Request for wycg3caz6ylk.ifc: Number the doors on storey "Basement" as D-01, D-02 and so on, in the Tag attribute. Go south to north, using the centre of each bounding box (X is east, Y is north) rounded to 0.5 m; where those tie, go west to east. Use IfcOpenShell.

First a look at what the model holds.

```python
import ifcopenshell
import ifcopenshell.util.element
import ifcopenshell.util.placement

model = ifcopenshell.open("wycg3caz6ylk.ifc")
print(model.schema)
storey = next(s for s in model.by_type("IfcBuildingStorey") if s.Name == "Basement")
doors = [e for e in ifcopenshell.util.element.get_decomposition(storey) if e.is_a("IfcDoor")]
for e in sorted(doors, key=lambda e: e.id()):
    origin = ifcopenshell.util.placement.get_local_placement(e.ObjectPlacement)[:3, 3]
    print(e.id(), e.Tag, e.Name, origin.round(2) + 0.0, sep=" | ")
```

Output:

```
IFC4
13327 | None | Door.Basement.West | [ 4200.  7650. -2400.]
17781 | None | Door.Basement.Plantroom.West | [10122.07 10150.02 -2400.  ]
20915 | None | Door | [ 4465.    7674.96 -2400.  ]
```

```python
import ifcopenshell
import ifcopenshell.geom
import ifcopenshell.util.element
import ifcopenshell.util.shape

model = ifcopenshell.open("wycg3caz6ylk.ifc")
settings = ifcopenshell.geom.settings()
settings.set("use-world-coords", True)


def centre(element):
    shape = ifcopenshell.geom.create_shape(settings, element)
    return ifcopenshell.util.shape.get_bbox_centroid(shape.geometry)


storey = next(s for s in model.by_type("IfcBuildingStorey") if s.Name == "Basement")
doors = [e for e in ifcopenshell.util.element.get_decomposition(storey) if e.is_a("IfcDoor")]

# Insertion points can sit at a corner or the storey origin, so sort by the geometry (in metres).
centres = {e: centre(e) for e in doors}
doors.sort(key=lambda e: (round(centres[e][1] / 0.5), centres[e][0]))

for i, e in enumerate(doors, start=1):
    number = f"D-{i:02d}"
    e.Tag = number
    print(e.id(), number)

model.write("wycg3caz6ylk_rev.ifc")
```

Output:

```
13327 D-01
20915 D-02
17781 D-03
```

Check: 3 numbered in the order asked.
